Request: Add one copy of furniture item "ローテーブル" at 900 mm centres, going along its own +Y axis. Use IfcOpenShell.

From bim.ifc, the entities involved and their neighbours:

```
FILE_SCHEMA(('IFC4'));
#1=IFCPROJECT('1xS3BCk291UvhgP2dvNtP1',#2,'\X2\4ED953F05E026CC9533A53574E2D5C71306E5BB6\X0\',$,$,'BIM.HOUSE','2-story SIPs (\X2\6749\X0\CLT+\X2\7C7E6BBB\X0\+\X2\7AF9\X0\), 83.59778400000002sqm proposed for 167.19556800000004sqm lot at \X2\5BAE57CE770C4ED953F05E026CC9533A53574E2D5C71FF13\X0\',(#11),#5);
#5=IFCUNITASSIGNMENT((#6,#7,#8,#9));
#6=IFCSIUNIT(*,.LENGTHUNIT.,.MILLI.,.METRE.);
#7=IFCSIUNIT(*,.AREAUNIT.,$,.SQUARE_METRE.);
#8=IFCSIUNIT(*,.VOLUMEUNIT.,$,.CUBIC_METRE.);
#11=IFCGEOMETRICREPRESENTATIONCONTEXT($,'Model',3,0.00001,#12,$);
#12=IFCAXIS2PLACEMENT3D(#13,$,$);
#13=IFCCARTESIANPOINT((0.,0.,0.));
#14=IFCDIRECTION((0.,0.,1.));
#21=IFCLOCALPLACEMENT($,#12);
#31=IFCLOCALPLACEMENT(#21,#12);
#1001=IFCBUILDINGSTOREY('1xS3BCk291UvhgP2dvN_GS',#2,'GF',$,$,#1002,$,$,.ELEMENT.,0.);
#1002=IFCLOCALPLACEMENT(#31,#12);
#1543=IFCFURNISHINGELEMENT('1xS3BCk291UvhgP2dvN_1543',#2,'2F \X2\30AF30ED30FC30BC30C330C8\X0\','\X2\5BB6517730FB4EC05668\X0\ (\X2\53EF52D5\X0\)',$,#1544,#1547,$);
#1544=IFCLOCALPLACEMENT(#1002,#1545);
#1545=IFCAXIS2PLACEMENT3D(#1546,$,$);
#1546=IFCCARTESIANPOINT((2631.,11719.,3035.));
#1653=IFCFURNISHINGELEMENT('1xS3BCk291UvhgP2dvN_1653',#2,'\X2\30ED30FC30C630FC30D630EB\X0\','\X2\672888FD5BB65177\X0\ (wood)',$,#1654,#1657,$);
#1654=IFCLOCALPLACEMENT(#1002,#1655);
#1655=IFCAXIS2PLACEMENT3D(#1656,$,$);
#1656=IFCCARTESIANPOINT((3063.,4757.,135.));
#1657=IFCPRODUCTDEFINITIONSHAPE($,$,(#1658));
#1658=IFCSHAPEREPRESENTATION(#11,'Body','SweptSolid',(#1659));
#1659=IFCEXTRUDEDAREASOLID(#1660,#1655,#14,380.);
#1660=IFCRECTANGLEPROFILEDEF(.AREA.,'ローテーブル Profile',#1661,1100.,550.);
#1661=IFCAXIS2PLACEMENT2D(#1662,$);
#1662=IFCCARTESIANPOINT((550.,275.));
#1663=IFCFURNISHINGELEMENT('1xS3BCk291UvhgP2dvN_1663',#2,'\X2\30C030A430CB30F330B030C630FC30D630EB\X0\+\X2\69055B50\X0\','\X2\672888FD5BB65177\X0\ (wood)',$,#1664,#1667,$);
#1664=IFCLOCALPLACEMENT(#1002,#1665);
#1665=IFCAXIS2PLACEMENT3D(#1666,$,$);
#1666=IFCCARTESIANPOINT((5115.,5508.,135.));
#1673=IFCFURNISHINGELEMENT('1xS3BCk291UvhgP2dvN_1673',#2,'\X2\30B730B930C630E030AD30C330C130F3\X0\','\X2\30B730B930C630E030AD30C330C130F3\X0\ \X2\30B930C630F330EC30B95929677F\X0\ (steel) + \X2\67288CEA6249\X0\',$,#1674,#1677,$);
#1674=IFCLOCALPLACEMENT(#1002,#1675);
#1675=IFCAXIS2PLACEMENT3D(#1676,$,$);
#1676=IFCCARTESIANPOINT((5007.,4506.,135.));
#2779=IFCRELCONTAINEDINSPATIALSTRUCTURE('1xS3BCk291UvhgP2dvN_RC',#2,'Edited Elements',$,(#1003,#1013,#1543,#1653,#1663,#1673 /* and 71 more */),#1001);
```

```python
import ifcopenshell
import ifcopenshell.api.geometry
import ifcopenshell.api.root
import ifcopenshell.util.element
import ifcopenshell.util.placement
import ifcopenshell.util.unit

model = ifcopenshell.open("bim.ifc")
unit_scale = ifcopenshell.util.unit.calculate_unit_scale(model)


def reuse_history(source, copy):
    """copy_class also copies each property set's owner history, people and application; keep the originals."""
    for rel in copy.IsDefinedBy:
        if rel.is_a("IfcRelDefinesByProperties") and (history := rel.RelatingPropertyDefinition.OwnerHistory):
            rel.RelatingPropertyDefinition.OwnerHistory = source.OwnerHistory
            ifcopenshell.util.element.remove_deep2(model, history)


source = model.by_guid("1xS3BCk291UvhgP2dvN_1653")
base = ifcopenshell.util.placement.get_local_placement(source.ObjectPlacement)
step = base[:3, 1] * 0.9 / unit_scale

for i in range(1, 2):
    copy = ifcopenshell.api.root.copy_class(model, product=source)
    copy.Representation = ifcopenshell.util.element.copy_deep(
        model, source.Representation, exclude=["IfcGeometricRepresentationContext", "IfcRepresentationMap"]
    )
    reuse_history(source, copy)
    matrix = base.copy()
    matrix[:3, 3] += i * step
    print("added at", matrix[:3, 3].round(3) + 0.0)
    ifcopenshell.api.geometry.edit_object_placement(model, product=copy, matrix=matrix, is_si=False)

model.write("bim-out.ifc")
```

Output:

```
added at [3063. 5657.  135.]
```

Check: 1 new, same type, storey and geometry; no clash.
